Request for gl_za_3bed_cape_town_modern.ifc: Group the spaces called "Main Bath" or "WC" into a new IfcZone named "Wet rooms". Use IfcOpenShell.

First a look at what the model holds.

```python
import ifcopenshell

model = ifcopenshell.open("gl_za_3bed_cape_town_modern.ifc")
print(model.schema)
seen = {}
for space in model.by_type("IfcSpace"):
    seen[space.LongName] = seen.get(space.LongName, 0) + 1
for name, count in sorted(seen.items(), key=str):
    print(count, "x", name)
print("zones:", [z.Name for z in model.by_type("IfcZone")][:20])
```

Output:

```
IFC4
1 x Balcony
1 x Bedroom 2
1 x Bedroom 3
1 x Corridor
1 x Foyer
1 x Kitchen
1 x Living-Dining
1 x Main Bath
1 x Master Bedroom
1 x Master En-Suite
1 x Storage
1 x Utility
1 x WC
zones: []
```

```python
import ifcopenshell
import ifcopenshell.api.group
import ifcopenshell.api.root

model = ifcopenshell.open("gl_za_3bed_cape_town_modern.ifc")

names = {"Main Bath", "WC"}
spaces = [s for s in model.by_type("IfcSpace") if s.LongName in names]

zone = ifcopenshell.api.root.create_entity(model, ifc_class="IfcZone", name="Wet rooms")
ifcopenshell.api.group.assign_group(model, products=spaces, group=zone)
print(len(spaces), "spaces in", zone.Name)

model.write("gl_za_3bed_cape_town_modern_updated.ifc")
```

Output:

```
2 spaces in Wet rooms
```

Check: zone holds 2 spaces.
